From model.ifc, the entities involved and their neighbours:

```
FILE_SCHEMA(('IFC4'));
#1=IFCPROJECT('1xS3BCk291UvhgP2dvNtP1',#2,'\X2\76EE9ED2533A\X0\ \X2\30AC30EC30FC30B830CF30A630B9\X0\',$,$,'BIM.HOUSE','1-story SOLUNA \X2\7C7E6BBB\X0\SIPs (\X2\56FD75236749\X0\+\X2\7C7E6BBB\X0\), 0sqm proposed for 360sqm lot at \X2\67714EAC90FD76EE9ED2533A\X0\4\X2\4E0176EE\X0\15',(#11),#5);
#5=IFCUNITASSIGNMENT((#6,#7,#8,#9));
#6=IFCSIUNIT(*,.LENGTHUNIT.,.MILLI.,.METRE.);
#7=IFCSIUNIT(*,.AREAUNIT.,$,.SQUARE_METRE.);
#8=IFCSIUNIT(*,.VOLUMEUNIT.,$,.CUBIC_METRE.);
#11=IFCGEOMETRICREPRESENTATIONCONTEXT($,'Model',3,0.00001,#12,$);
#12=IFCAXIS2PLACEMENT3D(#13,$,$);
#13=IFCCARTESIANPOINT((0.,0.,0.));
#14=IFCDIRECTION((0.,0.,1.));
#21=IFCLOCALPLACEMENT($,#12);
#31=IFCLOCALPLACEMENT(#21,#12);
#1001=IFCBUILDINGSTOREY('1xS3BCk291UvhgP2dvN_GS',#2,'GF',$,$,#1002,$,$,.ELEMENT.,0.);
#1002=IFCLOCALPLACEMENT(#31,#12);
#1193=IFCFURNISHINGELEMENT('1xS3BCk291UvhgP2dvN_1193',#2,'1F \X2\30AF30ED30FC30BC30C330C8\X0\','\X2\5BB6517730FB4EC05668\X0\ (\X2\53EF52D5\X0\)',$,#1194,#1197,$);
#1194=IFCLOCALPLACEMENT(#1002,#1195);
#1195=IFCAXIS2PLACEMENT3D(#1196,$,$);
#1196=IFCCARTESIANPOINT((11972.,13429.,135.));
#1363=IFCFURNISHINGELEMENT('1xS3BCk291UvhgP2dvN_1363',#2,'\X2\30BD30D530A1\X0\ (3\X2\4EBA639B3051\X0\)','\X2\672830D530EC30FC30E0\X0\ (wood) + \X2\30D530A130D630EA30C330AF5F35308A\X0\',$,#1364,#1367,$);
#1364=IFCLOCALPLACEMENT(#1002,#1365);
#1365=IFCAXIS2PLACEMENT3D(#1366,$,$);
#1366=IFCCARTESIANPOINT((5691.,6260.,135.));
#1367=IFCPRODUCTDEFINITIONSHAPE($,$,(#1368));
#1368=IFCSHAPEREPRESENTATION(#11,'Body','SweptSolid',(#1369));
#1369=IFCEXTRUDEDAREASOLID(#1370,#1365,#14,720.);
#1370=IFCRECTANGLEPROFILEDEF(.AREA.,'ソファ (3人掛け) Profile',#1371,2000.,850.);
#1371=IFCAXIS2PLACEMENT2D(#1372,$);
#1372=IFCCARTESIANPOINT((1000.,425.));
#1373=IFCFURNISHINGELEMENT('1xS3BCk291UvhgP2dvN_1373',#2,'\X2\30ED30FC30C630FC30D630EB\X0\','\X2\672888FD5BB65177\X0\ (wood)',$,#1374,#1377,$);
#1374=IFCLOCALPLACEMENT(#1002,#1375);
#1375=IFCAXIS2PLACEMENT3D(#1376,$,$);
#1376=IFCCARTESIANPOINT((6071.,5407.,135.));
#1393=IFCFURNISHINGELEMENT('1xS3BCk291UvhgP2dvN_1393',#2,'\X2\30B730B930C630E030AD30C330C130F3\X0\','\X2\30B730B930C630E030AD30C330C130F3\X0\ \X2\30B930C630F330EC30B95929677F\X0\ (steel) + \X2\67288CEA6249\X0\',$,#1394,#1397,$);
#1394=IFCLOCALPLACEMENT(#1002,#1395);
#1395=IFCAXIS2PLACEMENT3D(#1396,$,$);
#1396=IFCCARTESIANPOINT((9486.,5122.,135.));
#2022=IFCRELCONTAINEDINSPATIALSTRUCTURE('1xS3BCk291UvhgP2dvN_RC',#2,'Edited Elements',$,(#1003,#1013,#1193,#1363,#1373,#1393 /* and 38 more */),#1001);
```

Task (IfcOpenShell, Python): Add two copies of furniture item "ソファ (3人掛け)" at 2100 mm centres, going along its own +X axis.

```python
import ifcopenshell
import ifcopenshell.api.geometry
import ifcopenshell.api.root
import ifcopenshell.util.element
import ifcopenshell.util.placement
import ifcopenshell.util.unit

model = ifcopenshell.open("model.ifc")
unit_scale = ifcopenshell.util.unit.calculate_unit_scale(model)


def reuse_history(source, copy):
    """copy_class also copies each property set's owner history, people and application; keep the originals."""
    for rel in copy.IsDefinedBy:
        if rel.is_a("IfcRelDefinesByProperties") and (history := rel.RelatingPropertyDefinition.OwnerHistory):
            rel.RelatingPropertyDefinition.OwnerHistory = source.OwnerHistory
            ifcopenshell.util.element.remove_deep2(model, history)


source = model.by_guid("1xS3BCk291UvhgP2dvN_1363")
base = ifcopenshell.util.placement.get_local_placement(source.ObjectPlacement)
step = base[:3, 0] * 2.1 / unit_scale

for i in range(1, 3):
    copy = ifcopenshell.api.root.copy_class(model, product=source)
    copy.Representation = ifcopenshell.util.element.copy_deep(
        model, source.Representation, exclude=["IfcGeometricRepresentationContext", "IfcRepresentationMap"]
    )
    reuse_history(source, copy)
    matrix = base.copy()
    matrix[:3, 3] += i * step
    print("added at", matrix[:3, 3].round(3) + 0.0)
    ifcopenshell.api.geometry.edit_object_placement(model, product=copy, matrix=matrix, is_si=False)

model.write("model_rev.ifc")
```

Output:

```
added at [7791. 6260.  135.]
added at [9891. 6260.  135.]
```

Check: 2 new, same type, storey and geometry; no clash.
